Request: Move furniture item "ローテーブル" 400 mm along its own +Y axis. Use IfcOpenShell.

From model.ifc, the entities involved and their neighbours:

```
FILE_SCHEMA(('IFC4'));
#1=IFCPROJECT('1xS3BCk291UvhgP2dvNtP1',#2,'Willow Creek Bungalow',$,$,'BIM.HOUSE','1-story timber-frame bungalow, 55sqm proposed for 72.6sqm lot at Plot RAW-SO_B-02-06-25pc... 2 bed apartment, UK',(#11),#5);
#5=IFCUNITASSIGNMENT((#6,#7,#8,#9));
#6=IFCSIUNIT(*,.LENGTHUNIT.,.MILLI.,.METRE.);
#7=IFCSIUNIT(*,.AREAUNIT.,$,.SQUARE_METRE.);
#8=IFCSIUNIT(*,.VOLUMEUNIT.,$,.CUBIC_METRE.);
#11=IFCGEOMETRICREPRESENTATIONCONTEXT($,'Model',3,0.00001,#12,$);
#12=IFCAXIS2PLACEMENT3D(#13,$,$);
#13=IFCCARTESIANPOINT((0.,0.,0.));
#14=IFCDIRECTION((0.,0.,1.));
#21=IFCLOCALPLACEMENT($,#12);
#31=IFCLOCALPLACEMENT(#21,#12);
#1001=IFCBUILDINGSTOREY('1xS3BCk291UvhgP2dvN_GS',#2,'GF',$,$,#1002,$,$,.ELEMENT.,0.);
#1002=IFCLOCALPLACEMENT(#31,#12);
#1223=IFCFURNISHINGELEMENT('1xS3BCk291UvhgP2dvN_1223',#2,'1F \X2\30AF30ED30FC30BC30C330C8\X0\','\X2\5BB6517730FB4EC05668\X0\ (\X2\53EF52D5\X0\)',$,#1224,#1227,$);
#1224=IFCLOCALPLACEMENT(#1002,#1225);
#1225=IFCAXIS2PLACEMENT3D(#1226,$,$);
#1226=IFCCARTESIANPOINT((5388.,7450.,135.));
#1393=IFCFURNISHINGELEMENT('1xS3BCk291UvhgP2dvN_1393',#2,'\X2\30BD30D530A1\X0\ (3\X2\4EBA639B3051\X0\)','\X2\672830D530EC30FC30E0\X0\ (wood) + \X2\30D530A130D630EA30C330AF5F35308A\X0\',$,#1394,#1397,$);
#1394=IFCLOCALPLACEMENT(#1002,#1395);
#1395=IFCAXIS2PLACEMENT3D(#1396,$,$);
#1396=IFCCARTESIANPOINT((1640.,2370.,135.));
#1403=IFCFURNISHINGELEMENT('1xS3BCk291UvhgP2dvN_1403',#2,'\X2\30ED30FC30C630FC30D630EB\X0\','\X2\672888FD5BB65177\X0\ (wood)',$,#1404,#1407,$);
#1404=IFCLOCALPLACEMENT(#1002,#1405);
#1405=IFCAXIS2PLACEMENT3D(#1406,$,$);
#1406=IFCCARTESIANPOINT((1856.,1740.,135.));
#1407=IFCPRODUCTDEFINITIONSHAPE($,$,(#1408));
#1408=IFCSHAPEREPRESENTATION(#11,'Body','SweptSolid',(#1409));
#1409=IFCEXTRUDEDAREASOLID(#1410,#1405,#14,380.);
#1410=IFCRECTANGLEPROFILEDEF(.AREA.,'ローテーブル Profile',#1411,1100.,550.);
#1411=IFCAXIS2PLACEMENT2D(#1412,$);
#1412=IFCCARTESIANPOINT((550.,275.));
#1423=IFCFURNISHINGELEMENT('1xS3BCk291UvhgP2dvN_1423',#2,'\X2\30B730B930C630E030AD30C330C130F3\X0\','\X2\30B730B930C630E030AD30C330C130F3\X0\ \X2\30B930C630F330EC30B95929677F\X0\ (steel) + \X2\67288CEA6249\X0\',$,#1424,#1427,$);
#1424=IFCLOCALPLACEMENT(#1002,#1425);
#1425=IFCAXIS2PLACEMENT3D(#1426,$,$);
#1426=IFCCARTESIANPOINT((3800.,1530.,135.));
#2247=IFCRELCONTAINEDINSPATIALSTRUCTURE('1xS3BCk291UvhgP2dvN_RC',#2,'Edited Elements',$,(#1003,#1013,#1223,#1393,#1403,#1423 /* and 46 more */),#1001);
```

```python
import ifcopenshell
import ifcopenshell.api.geometry
import ifcopenshell.util.placement

model = ifcopenshell.open("model.ifc")

item = model.by_guid("1xS3BCk291UvhgP2dvN_1403")
matrix = ifcopenshell.util.placement.get_local_placement(item.ObjectPlacement)
matrix[:3, 3] += matrix[:3, 1] * 400.0
ifcopenshell.api.geometry.edit_object_placement(model, product=item, matrix=matrix, is_si=False)

print(ifcopenshell.util.placement.get_local_placement(item.ObjectPlacement).round(3) + 0.0)

model.write("model_v2.ifc")
```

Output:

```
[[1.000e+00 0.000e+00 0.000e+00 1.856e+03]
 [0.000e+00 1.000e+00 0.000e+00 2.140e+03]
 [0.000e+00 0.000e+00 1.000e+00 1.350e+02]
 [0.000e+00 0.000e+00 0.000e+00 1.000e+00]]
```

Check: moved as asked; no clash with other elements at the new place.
